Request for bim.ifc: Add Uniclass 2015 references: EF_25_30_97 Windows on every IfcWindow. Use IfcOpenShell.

First a look at what the model holds.

```python
import ifcopenshell

model = ifcopenshell.open("bim.ifc")
print(model.schema)
print("classifications:", [c.Name for c in model.by_type("IfcClassification")])
for ifc_class in ("IfcDoor", "IfcRoof", "IfcStair", "IfcWall", "IfcWindow"):
    print(ifc_class, len(model.by_type(ifc_class)))
```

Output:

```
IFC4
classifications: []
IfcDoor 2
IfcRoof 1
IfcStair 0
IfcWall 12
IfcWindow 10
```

```python
import ifcopenshell
import ifcopenshell.api.classification

model = ifcopenshell.open("bim.ifc")

system = ifcopenshell.api.classification.add_classification(model, classification="Uniclass 2015")

codes = {
    "IfcWindow": ("EF_25_30_97", "Windows"),
}
for ifc_class, (code, name) in codes.items():
    products = model.by_type(ifc_class)
    ifcopenshell.api.classification.add_reference(
        model, products=products, classification=system, identification=code, name=name
    )
    print(code, len(products))

model.write("bim_edited.ifc")
```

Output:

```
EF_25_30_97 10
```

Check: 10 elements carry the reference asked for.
